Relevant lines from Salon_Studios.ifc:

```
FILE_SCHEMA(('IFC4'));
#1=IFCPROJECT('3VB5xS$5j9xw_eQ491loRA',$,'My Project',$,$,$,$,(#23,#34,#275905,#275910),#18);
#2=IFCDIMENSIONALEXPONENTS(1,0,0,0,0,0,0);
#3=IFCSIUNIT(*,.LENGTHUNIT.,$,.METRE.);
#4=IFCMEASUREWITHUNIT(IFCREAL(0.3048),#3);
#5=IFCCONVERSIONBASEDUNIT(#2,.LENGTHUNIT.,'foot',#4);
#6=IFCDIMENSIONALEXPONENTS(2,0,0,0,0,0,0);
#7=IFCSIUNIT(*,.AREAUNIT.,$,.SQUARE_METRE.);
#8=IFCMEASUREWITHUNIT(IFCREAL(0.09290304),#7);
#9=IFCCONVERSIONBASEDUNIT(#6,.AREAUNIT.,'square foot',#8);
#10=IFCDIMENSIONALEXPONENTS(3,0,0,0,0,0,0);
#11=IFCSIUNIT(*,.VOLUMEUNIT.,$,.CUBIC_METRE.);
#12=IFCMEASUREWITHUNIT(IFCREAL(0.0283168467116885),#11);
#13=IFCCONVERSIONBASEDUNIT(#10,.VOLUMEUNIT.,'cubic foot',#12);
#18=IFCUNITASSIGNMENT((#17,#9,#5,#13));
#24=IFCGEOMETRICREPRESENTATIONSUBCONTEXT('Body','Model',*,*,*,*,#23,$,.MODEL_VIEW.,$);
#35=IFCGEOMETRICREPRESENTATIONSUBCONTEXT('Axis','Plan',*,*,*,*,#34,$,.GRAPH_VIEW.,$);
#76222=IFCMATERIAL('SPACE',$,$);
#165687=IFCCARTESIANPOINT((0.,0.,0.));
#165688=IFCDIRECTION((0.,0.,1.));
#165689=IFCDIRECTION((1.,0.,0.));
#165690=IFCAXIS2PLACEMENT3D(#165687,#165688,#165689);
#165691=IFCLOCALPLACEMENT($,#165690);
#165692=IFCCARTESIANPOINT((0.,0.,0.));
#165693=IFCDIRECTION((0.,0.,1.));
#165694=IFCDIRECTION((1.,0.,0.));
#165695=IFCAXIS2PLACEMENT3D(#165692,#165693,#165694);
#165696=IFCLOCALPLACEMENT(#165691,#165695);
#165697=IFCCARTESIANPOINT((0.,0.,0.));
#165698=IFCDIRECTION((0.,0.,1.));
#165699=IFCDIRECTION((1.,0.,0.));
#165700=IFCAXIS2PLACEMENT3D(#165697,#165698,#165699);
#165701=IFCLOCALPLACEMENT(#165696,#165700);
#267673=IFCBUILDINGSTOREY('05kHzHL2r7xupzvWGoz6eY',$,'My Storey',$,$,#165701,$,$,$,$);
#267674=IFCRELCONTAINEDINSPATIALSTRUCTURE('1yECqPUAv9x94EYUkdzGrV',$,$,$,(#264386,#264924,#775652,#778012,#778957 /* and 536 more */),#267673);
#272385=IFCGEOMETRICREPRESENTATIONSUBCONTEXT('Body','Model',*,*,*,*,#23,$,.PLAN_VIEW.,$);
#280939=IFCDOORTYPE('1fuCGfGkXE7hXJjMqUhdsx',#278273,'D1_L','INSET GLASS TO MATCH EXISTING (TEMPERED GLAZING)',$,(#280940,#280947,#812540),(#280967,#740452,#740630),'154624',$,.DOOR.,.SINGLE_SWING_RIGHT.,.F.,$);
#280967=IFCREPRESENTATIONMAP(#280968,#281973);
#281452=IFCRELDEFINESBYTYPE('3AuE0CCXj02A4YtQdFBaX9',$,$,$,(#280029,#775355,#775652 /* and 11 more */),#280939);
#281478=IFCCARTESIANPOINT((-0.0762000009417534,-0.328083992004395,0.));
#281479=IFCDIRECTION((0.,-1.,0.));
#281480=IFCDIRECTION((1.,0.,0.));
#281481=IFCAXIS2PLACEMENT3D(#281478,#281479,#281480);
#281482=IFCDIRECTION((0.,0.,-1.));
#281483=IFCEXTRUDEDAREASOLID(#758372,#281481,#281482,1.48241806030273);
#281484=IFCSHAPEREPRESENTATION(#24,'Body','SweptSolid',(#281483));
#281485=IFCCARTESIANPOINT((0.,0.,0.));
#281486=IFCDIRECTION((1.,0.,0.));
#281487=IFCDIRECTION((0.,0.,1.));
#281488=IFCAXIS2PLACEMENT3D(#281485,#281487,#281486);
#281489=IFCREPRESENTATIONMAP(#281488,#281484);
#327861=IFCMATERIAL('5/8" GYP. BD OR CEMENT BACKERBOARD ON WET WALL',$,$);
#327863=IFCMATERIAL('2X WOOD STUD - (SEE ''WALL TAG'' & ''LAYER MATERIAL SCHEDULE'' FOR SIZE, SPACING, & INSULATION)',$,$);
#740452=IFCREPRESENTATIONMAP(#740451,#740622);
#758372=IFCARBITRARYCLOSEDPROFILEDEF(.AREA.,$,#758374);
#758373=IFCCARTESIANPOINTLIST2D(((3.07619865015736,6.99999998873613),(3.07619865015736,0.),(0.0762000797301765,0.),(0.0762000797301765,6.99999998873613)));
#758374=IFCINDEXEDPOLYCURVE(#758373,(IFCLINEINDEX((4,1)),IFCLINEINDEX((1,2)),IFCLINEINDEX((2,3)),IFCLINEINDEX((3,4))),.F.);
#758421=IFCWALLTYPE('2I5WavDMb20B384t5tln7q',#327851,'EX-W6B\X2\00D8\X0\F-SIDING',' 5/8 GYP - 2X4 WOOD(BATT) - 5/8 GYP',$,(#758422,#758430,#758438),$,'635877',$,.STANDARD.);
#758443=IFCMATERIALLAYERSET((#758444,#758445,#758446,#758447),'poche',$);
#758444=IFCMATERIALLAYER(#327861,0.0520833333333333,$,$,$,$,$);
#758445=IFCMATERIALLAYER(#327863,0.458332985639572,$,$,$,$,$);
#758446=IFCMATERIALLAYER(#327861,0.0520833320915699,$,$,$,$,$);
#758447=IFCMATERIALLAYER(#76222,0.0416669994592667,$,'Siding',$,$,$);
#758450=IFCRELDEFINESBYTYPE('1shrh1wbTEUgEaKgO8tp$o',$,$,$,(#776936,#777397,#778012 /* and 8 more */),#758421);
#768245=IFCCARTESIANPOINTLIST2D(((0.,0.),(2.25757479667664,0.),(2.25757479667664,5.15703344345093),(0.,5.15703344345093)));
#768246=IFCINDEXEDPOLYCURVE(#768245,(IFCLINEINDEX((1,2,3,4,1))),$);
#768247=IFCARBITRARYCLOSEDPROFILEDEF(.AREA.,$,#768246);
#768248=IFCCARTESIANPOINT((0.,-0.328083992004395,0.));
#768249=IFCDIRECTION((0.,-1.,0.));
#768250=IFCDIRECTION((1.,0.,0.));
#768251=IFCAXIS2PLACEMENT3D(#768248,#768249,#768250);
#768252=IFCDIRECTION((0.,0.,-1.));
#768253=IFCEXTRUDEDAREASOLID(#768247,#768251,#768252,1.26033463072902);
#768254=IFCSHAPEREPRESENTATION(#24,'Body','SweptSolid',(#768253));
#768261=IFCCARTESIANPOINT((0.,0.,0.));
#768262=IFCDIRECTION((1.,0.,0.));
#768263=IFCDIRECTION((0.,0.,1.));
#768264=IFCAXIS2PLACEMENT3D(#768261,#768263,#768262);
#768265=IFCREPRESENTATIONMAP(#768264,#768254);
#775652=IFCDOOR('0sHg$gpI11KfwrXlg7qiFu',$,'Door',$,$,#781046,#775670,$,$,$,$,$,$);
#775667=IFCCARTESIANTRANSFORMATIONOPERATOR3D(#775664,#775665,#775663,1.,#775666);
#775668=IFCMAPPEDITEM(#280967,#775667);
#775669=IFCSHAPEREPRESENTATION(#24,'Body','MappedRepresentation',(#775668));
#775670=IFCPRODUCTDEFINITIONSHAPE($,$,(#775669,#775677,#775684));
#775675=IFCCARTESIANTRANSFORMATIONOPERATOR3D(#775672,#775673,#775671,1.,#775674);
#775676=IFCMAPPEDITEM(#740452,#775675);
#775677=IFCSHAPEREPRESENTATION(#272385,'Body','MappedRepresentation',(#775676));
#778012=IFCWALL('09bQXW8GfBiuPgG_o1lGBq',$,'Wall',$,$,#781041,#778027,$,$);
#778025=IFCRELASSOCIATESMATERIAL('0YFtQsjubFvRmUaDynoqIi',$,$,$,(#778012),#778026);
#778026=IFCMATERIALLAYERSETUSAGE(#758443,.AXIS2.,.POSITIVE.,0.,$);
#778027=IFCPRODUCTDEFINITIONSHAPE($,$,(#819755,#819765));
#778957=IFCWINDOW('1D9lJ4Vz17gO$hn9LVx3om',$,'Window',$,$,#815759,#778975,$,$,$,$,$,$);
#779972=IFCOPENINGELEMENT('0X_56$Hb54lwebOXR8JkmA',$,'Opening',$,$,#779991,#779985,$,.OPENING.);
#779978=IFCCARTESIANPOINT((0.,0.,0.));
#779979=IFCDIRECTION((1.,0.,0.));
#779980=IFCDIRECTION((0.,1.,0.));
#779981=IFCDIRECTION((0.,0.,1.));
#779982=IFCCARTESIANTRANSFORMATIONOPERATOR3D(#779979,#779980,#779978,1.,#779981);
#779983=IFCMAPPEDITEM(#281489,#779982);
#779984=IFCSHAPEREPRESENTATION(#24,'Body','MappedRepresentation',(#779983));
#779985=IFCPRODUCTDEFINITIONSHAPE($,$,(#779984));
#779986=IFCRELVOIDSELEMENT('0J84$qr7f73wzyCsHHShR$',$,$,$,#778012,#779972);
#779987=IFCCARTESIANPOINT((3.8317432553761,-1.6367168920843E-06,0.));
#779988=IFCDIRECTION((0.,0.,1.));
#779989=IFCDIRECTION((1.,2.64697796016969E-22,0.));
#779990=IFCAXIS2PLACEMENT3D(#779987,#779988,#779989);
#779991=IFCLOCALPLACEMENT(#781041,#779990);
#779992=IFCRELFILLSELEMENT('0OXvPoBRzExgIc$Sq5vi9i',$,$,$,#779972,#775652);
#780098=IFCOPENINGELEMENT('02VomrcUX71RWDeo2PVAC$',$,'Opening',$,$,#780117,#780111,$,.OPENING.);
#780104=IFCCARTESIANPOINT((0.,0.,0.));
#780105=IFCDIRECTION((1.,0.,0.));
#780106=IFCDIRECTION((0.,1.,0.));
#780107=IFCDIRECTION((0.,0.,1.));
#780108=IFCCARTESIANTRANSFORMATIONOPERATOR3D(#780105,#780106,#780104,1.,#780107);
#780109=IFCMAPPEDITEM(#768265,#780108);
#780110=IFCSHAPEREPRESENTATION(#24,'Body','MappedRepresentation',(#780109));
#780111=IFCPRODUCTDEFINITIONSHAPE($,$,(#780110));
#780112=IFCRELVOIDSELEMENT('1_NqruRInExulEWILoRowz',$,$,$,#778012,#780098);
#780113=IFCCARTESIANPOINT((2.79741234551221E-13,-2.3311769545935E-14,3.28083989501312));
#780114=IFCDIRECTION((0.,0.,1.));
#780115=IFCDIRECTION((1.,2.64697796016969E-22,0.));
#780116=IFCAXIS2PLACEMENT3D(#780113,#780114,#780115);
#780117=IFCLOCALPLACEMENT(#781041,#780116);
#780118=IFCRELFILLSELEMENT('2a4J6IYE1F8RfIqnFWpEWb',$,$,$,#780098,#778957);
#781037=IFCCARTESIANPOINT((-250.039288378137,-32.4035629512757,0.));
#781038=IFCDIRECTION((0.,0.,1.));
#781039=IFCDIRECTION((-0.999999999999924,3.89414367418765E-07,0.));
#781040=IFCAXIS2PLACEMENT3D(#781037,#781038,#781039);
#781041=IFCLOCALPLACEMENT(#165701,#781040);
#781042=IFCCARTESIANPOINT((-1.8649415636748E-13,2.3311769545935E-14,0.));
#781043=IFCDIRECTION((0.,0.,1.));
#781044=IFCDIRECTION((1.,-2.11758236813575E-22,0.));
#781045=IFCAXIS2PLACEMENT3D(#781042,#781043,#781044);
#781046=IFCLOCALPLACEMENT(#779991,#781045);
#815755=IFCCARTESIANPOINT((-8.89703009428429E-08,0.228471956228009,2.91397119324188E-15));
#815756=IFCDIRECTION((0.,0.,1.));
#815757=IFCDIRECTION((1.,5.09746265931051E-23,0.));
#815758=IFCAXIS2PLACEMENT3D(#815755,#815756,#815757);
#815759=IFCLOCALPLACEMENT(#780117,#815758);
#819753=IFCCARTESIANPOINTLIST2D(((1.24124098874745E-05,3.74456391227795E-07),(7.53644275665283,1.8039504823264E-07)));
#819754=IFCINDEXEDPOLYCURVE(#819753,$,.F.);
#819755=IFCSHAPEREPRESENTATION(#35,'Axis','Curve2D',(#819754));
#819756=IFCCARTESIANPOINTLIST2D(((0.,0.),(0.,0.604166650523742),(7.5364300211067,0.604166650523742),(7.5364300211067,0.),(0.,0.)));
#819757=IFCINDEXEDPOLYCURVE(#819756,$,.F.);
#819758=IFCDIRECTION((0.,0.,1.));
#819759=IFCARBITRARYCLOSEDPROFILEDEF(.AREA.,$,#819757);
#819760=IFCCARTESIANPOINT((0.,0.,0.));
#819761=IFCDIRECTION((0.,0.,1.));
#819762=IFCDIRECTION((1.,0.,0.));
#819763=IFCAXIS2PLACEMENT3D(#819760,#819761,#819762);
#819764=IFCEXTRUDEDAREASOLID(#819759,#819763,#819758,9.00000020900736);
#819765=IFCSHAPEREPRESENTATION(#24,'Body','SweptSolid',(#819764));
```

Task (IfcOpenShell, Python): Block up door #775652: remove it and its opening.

```python
import ifcopenshell
import ifcopenshell.api.feature
import ifcopenshell.api.root
import ifcopenshell.geom
import ifcopenshell.util.shape

model = ifcopenshell.open("Salon_Studios.ifc")
settings = ifcopenshell.geom.settings()


def volume(element):
    """Net volume in cubic metres, openings subtracted."""
    shape = ifcopenshell.geom.create_shape(settings, element)
    return ifcopenshell.util.shape.get_volume(shape.geometry)


door = model.by_id(775652)
opening = door.FillsVoids[0].RelatingOpeningElement
wall = opening.VoidsElements[0].RelatingBuildingElement
before = volume(wall)

ifcopenshell.api.root.remove_product(model, product=door)
ifcopenshell.api.feature.remove_feature(model, feature=opening)

after = volume(wall)

print(f"wall volume {before:.3f} -> {after:.3f} m3")

model.write("Salon_Studios-out.ifc")
```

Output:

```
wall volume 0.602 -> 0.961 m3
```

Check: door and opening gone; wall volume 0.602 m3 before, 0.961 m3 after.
